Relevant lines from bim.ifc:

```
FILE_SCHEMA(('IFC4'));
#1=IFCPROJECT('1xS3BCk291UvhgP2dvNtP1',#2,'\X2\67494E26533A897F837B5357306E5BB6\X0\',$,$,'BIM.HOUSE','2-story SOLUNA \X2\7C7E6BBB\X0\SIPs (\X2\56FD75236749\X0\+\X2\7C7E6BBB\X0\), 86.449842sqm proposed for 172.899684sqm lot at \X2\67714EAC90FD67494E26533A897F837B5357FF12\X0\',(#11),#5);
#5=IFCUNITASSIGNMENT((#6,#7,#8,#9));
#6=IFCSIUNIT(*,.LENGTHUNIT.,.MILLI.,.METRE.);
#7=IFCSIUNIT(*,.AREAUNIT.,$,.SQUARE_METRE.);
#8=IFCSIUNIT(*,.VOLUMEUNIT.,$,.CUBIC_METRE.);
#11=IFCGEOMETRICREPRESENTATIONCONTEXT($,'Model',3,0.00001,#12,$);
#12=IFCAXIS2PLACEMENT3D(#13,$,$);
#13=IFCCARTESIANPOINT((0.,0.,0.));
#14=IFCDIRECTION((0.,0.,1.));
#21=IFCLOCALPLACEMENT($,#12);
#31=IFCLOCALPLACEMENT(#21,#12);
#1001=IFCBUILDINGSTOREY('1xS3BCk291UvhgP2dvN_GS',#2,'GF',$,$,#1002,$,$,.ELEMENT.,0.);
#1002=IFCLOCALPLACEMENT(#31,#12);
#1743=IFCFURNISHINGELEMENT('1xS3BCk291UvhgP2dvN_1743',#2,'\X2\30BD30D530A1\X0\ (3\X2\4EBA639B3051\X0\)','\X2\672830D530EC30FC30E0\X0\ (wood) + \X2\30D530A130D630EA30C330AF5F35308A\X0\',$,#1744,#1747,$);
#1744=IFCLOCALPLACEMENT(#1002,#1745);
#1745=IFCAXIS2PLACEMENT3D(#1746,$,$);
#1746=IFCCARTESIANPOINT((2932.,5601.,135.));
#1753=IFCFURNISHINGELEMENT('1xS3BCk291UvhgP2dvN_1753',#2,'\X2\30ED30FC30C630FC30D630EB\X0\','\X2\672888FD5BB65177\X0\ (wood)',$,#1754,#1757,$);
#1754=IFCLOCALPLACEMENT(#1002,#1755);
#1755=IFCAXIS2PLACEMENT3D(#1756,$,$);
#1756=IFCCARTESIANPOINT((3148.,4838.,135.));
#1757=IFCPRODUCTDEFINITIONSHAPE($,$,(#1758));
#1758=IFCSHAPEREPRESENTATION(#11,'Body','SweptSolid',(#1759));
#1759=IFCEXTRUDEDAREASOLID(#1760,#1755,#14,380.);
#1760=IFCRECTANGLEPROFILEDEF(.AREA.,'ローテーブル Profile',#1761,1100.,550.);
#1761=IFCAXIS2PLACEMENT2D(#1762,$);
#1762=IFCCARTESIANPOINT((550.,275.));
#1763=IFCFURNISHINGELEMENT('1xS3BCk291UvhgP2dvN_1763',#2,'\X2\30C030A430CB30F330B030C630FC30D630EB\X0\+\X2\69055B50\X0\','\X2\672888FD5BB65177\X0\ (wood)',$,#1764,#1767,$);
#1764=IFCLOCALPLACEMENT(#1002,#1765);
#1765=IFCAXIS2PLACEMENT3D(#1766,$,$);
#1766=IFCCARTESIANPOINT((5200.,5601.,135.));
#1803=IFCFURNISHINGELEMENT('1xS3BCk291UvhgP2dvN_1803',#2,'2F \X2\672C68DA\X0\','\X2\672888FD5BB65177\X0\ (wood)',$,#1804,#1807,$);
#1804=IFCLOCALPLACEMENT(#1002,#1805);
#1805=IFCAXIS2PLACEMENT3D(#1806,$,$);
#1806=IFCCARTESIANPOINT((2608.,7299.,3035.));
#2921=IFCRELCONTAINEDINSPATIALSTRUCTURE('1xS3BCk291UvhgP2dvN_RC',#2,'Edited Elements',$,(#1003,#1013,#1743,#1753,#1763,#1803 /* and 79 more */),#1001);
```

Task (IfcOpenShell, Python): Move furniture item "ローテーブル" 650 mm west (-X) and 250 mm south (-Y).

```python
import ifcopenshell
import ifcopenshell.api.geometry
import ifcopenshell.util.placement

model = ifcopenshell.open("bim.ifc")

item = model.by_id(1753)
matrix = ifcopenshell.util.placement.get_local_placement(item.ObjectPlacement)
matrix[0, 3] -= 650.0
matrix[1, 3] -= 250.0
ifcopenshell.api.geometry.edit_object_placement(model, product=item, matrix=matrix, is_si=False)

print(ifcopenshell.util.placement.get_local_placement(item.ObjectPlacement).round(3) + 0.0)

model.write("bim_v2.ifc")
```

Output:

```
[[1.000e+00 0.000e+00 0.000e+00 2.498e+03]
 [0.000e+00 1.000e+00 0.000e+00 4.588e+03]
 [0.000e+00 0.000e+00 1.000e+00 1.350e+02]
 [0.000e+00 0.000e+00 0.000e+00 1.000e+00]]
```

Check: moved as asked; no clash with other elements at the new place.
